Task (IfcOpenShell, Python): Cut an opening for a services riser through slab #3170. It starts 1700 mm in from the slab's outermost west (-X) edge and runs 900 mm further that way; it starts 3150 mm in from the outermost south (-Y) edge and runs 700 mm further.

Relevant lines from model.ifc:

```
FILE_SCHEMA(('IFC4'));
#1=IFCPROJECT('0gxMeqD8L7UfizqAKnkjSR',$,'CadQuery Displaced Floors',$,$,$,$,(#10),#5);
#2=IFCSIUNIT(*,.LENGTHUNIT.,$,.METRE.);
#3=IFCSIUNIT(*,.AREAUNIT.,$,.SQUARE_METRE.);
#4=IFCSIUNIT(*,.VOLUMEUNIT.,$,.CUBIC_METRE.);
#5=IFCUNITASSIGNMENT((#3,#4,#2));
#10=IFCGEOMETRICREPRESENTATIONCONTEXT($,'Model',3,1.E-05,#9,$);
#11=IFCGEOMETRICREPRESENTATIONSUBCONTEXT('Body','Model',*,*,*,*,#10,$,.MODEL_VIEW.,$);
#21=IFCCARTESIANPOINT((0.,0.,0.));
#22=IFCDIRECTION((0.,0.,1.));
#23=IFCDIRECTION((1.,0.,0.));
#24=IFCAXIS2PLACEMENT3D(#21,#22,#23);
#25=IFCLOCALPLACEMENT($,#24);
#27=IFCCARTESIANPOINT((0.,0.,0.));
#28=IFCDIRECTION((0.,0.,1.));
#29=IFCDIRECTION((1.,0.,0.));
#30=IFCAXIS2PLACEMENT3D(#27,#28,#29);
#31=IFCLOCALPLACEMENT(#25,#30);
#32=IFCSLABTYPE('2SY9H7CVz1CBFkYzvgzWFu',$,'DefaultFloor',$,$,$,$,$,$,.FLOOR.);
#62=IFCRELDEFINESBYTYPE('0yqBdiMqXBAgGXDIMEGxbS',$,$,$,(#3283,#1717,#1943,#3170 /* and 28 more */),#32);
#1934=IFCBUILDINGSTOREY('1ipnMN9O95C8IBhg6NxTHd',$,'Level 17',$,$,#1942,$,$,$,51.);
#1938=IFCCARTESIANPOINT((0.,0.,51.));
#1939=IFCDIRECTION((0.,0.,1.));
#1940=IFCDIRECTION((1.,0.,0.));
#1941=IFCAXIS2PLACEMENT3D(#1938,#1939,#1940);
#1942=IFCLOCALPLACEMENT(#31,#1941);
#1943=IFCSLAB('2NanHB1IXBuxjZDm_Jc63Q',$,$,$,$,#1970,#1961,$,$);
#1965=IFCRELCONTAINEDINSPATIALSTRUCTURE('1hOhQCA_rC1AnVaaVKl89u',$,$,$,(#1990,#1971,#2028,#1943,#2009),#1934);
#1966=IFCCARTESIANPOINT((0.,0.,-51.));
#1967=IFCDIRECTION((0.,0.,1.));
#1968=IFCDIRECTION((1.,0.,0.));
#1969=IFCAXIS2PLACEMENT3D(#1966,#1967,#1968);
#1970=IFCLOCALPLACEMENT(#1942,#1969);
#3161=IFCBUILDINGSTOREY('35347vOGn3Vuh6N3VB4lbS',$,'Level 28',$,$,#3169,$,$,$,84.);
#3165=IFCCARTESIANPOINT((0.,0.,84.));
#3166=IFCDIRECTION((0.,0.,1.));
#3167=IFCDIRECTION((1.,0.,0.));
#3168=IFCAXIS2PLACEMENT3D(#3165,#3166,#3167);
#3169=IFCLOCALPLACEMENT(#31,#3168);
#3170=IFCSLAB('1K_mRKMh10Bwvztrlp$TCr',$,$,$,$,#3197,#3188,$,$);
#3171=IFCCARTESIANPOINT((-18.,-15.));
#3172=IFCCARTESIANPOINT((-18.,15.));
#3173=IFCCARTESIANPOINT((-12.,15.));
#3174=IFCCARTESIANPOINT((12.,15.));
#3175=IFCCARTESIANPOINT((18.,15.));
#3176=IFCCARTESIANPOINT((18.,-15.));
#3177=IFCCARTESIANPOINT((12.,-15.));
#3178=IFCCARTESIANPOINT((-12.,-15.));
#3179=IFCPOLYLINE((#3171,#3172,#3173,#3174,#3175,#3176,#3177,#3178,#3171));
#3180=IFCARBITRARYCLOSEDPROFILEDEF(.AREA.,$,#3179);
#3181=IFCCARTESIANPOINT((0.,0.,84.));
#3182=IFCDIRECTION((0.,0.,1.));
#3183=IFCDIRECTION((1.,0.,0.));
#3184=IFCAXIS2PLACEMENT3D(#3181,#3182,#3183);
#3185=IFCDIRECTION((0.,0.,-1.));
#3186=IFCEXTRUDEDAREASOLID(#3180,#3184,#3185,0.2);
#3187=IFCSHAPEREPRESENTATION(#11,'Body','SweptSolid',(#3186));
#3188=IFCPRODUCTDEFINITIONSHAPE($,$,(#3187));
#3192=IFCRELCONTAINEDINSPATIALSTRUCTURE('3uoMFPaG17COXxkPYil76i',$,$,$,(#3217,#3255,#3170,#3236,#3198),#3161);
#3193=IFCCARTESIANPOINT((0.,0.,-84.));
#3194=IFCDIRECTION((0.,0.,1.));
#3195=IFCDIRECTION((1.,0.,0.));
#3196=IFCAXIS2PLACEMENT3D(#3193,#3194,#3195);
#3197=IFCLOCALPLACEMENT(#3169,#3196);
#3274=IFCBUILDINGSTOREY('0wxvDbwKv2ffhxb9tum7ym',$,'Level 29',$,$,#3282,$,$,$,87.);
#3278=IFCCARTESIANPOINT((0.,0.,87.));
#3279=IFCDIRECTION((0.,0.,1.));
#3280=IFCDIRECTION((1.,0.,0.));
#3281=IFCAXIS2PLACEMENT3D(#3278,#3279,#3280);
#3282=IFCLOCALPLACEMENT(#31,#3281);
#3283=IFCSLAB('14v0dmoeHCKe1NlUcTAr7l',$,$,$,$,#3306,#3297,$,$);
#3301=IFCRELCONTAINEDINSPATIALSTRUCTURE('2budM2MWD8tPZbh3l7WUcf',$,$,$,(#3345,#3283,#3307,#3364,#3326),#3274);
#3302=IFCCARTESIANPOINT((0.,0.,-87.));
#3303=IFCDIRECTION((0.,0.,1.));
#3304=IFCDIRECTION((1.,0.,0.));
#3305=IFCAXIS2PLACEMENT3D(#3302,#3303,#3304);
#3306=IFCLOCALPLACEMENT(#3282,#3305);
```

```python
import numpy as np
import ifcopenshell
import ifcopenshell.api.feature
import ifcopenshell.api.geometry
import ifcopenshell.api.root
import ifcopenshell.geom
import ifcopenshell.util.placement
import ifcopenshell.util.representation
import ifcopenshell.util.shape
import ifcopenshell.util.unit

model = ifcopenshell.open("model.ifc")
unit_scale = ifcopenshell.util.unit.calculate_unit_scale(model)
settings = ifcopenshell.geom.settings()


def volume(element):
    """Net volume in cubic metres, openings subtracted."""
    shape = ifcopenshell.geom.create_shape(settings, element)
    return ifcopenshell.util.shape.get_volume(shape.geometry)


slab = model.by_guid("1K_mRKMh10Bwvztrlp$TCr")
before = volume(slab)

# Extent in the slab's own axes, in metres. The edges named are its -X and -Y sides.
slab_shape = ifcopenshell.geom.create_shape(settings, slab)
vertices = ifcopenshell.util.shape.get_vertices(slab_shape.geometry)
x_min, y_min, bottom = vertices.min(axis=0)
top = vertices[:, 2].max()

opening = ifcopenshell.api.root.create_entity(model, ifc_class="IfcOpeningElement", name="Services riser opening", predefined_type="OPENING")
context = ifcopenshell.util.representation.get_context(model, "Model", "Body", "MODEL_VIEW")
width, depth = 0.9, 0.7
outline = [(0.0, 0.0), (width, 0.0), (width, depth), (0.0, depth), (0.0, 0.0)]
# Overshoot both faces by 50 mm so the cut is clean.
shape = ifcopenshell.api.geometry.add_slab_representation(
    model, context=context, depth=top - bottom + 0.1, polyline=outline
)
ifcopenshell.api.geometry.assign_representation(model, product=opening, representation=shape)

matrix = ifcopenshell.util.placement.get_local_placement(slab.ObjectPlacement)
matrix[:, 3] = matrix @ np.append(np.array([x_min + 1.7, y_min + 3.15, bottom - 0.05]) / unit_scale, 1.0)
ifcopenshell.api.geometry.edit_object_placement(model, product=opening, matrix=matrix, is_si=False)
ifcopenshell.api.feature.add_feature(model, feature=opening, element=slab)

after = volume(slab)

print(f"slab volume {before:.3f} -> {after:.3f} m3")

model.write("model_edited.ifc")
```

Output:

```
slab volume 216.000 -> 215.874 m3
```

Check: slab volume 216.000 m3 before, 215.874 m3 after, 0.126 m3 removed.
